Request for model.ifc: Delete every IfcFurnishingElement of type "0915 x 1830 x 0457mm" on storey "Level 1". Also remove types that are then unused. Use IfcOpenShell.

First a look at what the model holds.

```python
import ifcopenshell
import ifcopenshell.util.element

model = ifcopenshell.open("model.ifc")
print(model.schema)
storey = next(s for s in model.by_type("IfcBuildingStorey") if s.Name == "Level 1")
furniture = [e for e in ifcopenshell.util.element.get_decomposition(storey) if e.is_a("IfcFurnishingElement")]
seen = {}
for e in furniture:
    element_type = ifcopenshell.util.element.get_type(e)
    name = element_type.Name if element_type not in (None, e) else None
    seen[name] = seen.get(name, 0) + 1
for name, count in sorted(seen.items(), key=str):
    print(count, "x", name)
```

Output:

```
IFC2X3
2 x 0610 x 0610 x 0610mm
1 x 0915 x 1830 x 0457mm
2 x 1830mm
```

```python
import ifcopenshell
import ifcopenshell.api.root
import ifcopenshell.util.element

model = ifcopenshell.open("model.ifc")

storey = next(s for s in model.by_type("IfcBuildingStorey") if s.Name == "Level 1")
furniture = [e for e in ifcopenshell.util.element.get_decomposition(storey) if e.is_a("IfcFurnishingElement")]
targets = [e for e in furniture if (t := ifcopenshell.util.element.get_type(e)) not in (None, e) and t.Name == "0915 x 1830 x 0457mm"]
types = {ifcopenshell.util.element.get_type(e) for e in targets} - {None, *targets}

for e in targets:
    ifcopenshell.api.root.remove_product(model, product=e)
print(len(targets), "removed")

unused = [t for t in types if not ifcopenshell.util.element.get_types(t)]
for t in unused:
    ifcopenshell.api.root.remove_product(model, product=t)
print(len(unused), "unused types removed")

model.write("model-out.ifc")
```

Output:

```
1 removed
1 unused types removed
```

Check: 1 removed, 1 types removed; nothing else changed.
